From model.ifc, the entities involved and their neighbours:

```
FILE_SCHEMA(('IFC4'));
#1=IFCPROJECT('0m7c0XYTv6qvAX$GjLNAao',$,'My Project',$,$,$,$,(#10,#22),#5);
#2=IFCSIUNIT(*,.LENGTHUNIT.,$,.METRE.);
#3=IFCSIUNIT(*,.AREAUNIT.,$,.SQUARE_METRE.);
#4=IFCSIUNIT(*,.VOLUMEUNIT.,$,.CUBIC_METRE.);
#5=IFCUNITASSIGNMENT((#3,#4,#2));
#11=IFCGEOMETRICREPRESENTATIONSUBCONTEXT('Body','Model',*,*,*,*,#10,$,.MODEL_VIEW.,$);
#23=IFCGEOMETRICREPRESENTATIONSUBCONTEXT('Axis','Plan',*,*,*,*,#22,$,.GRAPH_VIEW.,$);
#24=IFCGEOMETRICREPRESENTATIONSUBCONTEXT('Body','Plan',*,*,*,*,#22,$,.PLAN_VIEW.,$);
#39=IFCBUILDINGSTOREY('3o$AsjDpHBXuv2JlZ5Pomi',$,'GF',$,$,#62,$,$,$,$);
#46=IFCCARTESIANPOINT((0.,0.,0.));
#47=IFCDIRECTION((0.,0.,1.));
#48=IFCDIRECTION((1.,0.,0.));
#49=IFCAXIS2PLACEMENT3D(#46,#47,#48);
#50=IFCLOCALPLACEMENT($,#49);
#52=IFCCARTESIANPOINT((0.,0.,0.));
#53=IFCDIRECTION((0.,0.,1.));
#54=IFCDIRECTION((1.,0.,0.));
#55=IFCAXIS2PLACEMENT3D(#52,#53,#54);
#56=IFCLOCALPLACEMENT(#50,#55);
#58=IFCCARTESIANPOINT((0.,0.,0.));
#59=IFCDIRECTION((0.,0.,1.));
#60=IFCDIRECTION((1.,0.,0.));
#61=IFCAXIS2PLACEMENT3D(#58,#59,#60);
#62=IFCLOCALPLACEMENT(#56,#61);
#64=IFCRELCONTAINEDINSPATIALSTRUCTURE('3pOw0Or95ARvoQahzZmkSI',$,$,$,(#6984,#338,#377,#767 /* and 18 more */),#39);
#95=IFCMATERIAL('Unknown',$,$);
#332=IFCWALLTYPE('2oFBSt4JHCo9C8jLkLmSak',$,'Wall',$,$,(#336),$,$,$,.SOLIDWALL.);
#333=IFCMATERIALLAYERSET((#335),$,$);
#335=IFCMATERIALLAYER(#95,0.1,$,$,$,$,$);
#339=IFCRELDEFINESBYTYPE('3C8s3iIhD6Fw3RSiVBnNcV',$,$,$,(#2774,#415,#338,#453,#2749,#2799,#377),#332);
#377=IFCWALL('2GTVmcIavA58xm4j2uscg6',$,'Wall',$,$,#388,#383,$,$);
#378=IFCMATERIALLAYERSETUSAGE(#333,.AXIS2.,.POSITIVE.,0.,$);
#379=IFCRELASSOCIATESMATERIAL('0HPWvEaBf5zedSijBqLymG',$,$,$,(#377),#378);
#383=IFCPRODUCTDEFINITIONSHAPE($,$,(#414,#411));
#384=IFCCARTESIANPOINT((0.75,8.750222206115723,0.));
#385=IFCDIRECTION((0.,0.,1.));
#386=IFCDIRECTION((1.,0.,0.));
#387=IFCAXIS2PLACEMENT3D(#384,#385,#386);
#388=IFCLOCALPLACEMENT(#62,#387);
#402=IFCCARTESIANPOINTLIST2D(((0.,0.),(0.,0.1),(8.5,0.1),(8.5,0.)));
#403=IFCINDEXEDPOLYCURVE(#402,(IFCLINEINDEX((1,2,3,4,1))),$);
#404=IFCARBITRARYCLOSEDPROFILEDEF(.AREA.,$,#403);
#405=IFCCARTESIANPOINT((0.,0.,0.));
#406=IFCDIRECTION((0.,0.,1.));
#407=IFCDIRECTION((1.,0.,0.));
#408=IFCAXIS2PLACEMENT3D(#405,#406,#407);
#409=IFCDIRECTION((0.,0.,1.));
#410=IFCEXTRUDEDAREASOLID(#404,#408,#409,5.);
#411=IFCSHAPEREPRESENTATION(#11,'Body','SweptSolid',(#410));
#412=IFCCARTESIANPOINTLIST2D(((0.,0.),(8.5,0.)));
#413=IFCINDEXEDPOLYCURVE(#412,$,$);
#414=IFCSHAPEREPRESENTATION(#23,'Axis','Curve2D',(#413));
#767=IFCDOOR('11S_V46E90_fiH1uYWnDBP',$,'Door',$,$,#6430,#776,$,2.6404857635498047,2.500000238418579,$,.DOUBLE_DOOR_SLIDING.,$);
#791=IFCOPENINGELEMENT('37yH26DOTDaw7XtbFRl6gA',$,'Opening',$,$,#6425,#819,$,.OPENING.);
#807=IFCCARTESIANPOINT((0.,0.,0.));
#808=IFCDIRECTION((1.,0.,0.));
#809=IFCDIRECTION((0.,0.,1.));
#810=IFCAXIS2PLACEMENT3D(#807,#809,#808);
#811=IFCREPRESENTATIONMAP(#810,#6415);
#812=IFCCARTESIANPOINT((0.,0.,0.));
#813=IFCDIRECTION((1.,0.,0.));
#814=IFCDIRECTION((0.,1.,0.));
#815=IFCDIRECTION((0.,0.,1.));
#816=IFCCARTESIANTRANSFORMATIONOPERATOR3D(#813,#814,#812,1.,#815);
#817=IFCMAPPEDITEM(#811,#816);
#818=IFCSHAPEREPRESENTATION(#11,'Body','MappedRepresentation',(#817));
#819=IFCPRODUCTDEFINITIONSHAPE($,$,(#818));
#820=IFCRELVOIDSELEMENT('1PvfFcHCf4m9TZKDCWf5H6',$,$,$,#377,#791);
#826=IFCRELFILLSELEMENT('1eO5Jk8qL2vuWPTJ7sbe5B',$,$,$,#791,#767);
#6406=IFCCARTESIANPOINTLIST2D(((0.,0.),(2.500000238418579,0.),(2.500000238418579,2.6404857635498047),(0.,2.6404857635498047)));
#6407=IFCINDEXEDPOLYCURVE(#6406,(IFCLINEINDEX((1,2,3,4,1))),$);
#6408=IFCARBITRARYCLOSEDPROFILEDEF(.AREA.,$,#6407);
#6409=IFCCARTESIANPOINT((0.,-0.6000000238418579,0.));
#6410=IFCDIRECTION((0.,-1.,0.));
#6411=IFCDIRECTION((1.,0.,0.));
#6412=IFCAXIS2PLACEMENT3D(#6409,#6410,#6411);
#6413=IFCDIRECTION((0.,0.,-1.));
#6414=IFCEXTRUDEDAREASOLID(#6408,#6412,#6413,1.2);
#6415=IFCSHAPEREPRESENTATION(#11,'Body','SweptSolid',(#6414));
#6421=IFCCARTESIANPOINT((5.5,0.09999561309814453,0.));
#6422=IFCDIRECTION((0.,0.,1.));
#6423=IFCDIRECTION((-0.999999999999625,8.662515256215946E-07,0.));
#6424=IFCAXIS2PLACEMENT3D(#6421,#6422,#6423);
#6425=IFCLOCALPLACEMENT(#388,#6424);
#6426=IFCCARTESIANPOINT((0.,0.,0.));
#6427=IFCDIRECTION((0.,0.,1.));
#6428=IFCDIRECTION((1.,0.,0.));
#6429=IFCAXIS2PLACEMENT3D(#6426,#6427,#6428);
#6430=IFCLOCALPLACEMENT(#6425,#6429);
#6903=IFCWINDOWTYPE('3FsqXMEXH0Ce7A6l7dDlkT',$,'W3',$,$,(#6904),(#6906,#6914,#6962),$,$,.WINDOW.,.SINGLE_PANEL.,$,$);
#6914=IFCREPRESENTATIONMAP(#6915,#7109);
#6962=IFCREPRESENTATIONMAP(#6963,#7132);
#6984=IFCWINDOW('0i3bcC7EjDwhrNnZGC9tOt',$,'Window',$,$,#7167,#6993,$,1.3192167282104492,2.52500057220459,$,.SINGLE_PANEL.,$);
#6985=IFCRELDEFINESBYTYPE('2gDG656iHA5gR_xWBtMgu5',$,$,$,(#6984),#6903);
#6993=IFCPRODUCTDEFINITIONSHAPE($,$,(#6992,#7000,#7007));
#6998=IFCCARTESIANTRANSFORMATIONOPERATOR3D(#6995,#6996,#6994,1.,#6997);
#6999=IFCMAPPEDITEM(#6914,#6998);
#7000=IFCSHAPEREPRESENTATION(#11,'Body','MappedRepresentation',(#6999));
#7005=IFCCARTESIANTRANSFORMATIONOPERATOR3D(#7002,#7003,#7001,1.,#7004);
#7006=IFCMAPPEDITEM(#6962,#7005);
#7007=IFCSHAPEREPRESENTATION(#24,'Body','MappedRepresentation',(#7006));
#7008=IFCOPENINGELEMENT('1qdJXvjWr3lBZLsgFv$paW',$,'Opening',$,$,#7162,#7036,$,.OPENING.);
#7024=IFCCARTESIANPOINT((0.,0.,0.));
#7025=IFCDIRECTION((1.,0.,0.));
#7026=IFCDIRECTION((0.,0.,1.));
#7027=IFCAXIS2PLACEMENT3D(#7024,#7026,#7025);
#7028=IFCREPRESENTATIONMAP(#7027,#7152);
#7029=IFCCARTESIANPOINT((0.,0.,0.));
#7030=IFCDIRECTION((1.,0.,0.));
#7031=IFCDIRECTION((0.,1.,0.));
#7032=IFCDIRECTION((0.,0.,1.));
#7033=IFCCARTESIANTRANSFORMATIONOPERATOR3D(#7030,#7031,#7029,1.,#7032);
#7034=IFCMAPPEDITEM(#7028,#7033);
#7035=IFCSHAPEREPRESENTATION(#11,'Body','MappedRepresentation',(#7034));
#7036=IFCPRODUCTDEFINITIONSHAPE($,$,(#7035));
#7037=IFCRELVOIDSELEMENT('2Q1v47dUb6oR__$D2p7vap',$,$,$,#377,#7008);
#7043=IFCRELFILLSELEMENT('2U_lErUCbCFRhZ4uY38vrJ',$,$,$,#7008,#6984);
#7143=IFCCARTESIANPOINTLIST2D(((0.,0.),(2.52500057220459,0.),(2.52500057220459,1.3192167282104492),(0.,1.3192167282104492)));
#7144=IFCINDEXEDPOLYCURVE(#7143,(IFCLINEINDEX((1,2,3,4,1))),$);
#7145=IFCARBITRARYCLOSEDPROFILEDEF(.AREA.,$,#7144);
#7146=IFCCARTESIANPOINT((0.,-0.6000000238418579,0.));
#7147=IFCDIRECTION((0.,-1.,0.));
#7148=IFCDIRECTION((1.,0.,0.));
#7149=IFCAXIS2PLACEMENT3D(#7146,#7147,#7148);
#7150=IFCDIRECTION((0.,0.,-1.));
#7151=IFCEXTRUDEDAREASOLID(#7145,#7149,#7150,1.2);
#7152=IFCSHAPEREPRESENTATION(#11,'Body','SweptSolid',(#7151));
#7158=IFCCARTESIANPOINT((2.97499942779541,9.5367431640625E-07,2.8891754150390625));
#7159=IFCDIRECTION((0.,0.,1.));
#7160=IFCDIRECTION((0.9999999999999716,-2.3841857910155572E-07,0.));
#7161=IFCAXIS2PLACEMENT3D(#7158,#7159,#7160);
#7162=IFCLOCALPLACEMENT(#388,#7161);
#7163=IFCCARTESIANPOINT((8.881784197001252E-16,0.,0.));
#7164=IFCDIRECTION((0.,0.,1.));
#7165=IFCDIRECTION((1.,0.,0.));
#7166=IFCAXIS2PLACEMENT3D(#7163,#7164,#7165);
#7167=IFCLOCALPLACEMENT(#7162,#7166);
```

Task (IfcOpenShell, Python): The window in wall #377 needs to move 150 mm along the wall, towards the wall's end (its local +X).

```python
import ifcopenshell
import ifcopenshell.api.geometry
import ifcopenshell.util.placement
import ifcopenshell.util.unit

model = ifcopenshell.open("model.ifc")
unit_scale = ifcopenshell.util.unit.calculate_unit_scale(model)

window = model.by_guid("0i3bcC7EjDwhrNnZGC9tOt")
opening = window.FillsVoids[0].RelatingOpeningElement
wall = opening.VoidsElements[0].RelatingBuildingElement

wall_matrix = ifcopenshell.util.placement.get_local_placement(wall.ObjectPlacement)
shift = wall_matrix[:3, 0] * 0.15 / unit_scale
before = ifcopenshell.util.placement.get_local_placement(window.ObjectPlacement)[:3, 3].copy()

# The window is placed relative to its opening, so it follows when the opening moves.
matrix = ifcopenshell.util.placement.get_local_placement(opening.ObjectPlacement)
matrix[:3, 3] += shift
ifcopenshell.api.geometry.edit_object_placement(
    model, product=opening, matrix=matrix, is_si=False, should_transform_children=True
)

after = ifcopenshell.util.placement.get_local_placement(window.ObjectPlacement)[:3, 3]
print("window moved by", (after - before).round(3) + 0.0)

model.write("model-out.ifc")
```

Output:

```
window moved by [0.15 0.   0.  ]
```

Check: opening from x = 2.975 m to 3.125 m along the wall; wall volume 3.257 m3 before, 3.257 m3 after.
